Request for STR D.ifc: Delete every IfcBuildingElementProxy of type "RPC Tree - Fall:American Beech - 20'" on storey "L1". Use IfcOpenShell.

First a look at what the model holds.

```python
import ifcopenshell
import ifcopenshell.util.element

model = ifcopenshell.open("STR D.ifc")
print(model.schema)
storey = next(s for s in model.by_type("IfcBuildingStorey") if s.Name == "L1")
proxies = [e for e in ifcopenshell.util.element.get_decomposition(storey) if e.is_a("IfcBuildingElementProxy")]
seen = {}
for e in proxies:
    element_type = ifcopenshell.util.element.get_type(e)
    name = element_type.Name if element_type not in (None, e) else None
    seen[name] = seen.get(name, 0) + 1
for name, count in sorted(seen.items(), key=str):
    print(count, "x", name)
```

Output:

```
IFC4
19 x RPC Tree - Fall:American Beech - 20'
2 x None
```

```python
import ifcopenshell
import ifcopenshell.api.root
import ifcopenshell.util.element

model = ifcopenshell.open("STR D.ifc")

storey = next(s for s in model.by_type("IfcBuildingStorey") if s.Name == "L1")
proxies = [e for e in ifcopenshell.util.element.get_decomposition(storey) if e.is_a("IfcBuildingElementProxy")]
targets = [e for e in proxies if (t := ifcopenshell.util.element.get_type(e)) not in (None, e) and t.Name == "RPC Tree - Fall:American Beech - 20'"]

for e in targets:
    ifcopenshell.api.root.remove_product(model, product=e)
print(len(targets), "removed")

model.write("STR D_edited.ifc")
```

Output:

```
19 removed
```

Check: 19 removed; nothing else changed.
